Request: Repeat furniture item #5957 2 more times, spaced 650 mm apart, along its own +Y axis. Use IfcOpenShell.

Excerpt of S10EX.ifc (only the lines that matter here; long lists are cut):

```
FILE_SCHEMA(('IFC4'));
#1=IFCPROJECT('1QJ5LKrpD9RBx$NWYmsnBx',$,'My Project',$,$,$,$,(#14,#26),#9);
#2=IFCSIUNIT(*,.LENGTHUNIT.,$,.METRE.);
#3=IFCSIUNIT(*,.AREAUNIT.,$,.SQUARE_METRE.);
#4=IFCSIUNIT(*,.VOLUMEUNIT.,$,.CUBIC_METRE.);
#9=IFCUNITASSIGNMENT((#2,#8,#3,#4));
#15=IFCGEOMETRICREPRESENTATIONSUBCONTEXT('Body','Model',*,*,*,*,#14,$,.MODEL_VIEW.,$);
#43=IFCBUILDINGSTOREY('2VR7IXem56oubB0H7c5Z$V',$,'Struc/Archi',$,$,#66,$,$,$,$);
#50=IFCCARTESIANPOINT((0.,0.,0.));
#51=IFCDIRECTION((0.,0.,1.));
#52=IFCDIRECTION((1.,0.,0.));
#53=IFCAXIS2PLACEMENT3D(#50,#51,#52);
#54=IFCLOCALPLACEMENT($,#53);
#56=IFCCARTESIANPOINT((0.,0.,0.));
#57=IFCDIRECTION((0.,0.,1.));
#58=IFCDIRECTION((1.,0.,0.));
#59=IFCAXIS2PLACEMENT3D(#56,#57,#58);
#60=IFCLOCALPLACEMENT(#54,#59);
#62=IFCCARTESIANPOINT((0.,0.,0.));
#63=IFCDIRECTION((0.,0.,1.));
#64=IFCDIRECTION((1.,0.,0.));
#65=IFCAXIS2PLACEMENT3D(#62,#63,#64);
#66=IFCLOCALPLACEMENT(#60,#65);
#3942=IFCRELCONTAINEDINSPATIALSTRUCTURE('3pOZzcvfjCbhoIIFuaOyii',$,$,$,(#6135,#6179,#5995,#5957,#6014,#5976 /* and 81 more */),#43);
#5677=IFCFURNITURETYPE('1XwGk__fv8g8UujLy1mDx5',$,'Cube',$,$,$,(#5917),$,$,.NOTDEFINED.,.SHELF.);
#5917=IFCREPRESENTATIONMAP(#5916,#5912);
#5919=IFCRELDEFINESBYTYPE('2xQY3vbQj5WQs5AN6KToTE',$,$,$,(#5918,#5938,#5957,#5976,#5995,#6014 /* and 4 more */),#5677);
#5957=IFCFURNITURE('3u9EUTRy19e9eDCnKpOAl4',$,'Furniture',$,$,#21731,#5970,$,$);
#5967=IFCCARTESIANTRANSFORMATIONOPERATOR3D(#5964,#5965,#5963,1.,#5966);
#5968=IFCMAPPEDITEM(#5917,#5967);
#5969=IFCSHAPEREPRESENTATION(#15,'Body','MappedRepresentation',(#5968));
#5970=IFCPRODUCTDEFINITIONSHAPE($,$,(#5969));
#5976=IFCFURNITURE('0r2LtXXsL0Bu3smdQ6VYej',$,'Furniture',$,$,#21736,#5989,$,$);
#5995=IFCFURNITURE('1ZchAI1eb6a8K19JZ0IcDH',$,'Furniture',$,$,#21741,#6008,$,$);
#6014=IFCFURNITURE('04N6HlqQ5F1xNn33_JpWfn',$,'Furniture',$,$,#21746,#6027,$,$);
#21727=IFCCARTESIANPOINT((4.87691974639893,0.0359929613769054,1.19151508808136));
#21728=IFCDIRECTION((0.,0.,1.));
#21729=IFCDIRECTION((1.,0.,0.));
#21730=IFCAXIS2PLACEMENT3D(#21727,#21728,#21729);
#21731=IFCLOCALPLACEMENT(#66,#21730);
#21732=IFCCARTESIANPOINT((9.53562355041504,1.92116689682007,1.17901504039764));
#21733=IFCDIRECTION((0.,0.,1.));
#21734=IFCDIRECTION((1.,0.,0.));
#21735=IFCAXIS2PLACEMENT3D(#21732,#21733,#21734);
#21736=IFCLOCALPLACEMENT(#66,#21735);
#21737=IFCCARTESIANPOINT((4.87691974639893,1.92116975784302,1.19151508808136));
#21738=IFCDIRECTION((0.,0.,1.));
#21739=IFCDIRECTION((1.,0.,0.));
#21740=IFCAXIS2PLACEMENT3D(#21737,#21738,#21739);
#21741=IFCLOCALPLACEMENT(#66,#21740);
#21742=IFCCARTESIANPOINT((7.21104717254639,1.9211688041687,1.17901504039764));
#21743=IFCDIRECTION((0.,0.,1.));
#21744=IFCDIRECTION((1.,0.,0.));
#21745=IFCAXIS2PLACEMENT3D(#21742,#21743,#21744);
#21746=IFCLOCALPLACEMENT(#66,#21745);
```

```python
import ifcopenshell
import ifcopenshell.api.geometry
import ifcopenshell.api.root
import ifcopenshell.util.element
import ifcopenshell.util.placement

model = ifcopenshell.open("S10EX.ifc")

source = model.by_id(5957)
base = ifcopenshell.util.placement.get_local_placement(source.ObjectPlacement)
step = base[:3, 1] * 0.65

for i in range(1, 3):
    copy = ifcopenshell.api.root.copy_class(model, product=source)
    copy.Representation = ifcopenshell.util.element.copy_deep(
        model, source.Representation, exclude=["IfcGeometricRepresentationContext", "IfcRepresentationMap"]
    )
    matrix = base.copy()
    matrix[:3, 3] += i * step
    print("added at", matrix[:3, 3].round(3) + 0.0)
    ifcopenshell.api.geometry.edit_object_placement(model, product=copy, matrix=matrix, is_si=False)

model.write("S10EX_updated.ifc")
```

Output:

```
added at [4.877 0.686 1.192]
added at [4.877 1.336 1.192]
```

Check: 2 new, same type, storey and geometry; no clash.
